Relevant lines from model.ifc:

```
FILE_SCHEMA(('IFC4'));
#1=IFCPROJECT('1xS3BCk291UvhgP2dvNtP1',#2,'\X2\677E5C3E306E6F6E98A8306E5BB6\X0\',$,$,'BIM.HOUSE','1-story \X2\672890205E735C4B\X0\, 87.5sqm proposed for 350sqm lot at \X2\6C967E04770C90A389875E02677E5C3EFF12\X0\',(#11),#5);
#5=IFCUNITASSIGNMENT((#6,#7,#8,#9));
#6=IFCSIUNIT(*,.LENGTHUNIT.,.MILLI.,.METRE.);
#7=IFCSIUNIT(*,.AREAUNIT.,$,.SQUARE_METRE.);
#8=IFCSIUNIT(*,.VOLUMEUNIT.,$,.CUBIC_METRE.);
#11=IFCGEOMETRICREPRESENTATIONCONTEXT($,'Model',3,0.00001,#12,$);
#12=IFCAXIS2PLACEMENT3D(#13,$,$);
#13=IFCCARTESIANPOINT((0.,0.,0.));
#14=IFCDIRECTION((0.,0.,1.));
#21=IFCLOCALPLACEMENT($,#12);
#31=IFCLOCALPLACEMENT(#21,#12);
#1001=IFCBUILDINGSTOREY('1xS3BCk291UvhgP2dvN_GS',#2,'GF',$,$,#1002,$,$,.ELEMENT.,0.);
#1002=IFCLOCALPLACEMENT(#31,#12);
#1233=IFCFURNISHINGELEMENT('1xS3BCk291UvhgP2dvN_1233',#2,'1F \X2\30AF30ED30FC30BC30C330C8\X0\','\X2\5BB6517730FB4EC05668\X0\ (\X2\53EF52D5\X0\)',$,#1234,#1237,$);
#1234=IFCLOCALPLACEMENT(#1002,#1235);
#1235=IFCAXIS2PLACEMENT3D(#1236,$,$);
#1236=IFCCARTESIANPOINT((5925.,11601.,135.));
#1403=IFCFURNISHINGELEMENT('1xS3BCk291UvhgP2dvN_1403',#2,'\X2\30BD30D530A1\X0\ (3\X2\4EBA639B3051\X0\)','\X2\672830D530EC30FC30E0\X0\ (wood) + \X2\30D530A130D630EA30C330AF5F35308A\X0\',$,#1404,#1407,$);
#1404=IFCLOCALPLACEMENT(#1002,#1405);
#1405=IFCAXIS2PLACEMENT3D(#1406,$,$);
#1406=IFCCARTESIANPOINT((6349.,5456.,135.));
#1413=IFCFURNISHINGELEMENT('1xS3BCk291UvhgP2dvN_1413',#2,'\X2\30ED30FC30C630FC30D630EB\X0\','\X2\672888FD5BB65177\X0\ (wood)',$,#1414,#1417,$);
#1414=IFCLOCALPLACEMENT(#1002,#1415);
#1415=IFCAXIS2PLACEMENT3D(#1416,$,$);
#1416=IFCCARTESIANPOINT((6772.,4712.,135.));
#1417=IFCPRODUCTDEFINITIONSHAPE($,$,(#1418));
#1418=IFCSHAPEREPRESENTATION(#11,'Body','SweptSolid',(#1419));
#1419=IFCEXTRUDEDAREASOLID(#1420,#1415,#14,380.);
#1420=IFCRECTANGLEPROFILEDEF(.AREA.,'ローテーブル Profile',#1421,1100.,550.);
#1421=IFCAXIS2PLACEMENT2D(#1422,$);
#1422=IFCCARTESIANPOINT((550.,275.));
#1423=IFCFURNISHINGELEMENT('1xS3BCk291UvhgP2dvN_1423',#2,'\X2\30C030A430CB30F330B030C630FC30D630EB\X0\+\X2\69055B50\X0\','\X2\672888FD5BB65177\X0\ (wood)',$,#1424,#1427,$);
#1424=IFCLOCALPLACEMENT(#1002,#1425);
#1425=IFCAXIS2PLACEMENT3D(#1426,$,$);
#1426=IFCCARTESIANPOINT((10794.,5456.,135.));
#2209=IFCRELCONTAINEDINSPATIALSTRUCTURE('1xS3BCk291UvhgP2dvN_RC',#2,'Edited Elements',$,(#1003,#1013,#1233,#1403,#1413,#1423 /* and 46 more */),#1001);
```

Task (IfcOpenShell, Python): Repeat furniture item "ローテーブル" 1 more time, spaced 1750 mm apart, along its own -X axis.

```python
import ifcopenshell
import ifcopenshell.api.geometry
import ifcopenshell.api.root
import ifcopenshell.util.element
import ifcopenshell.util.placement
import ifcopenshell.util.unit

model = ifcopenshell.open("model.ifc")
unit_scale = ifcopenshell.util.unit.calculate_unit_scale(model)


def reuse_history(source, copy):
    """copy_class also copies each property set's owner history, people and application; keep the originals."""
    for rel in copy.IsDefinedBy:
        if rel.is_a("IfcRelDefinesByProperties") and (history := rel.RelatingPropertyDefinition.OwnerHistory):
            rel.RelatingPropertyDefinition.OwnerHistory = source.OwnerHistory
            ifcopenshell.util.element.remove_deep2(model, history)


source = model.by_guid("1xS3BCk291UvhgP2dvN_1413")
base = ifcopenshell.util.placement.get_local_placement(source.ObjectPlacement)
step = -base[:3, 0] * 1.75 / unit_scale

for i in range(1, 2):
    copy = ifcopenshell.api.root.copy_class(model, product=source)
    copy.Representation = ifcopenshell.util.element.copy_deep(
        model, source.Representation, exclude=["IfcGeometricRepresentationContext", "IfcRepresentationMap"]
    )
    reuse_history(source, copy)
    matrix = base.copy()
    matrix[:3, 3] += i * step
    print("added at", matrix[:3, 3].round(3) + 0.0)
    ifcopenshell.api.geometry.edit_object_placement(model, product=copy, matrix=matrix, is_si=False)

model.write("model_edited.ifc")
```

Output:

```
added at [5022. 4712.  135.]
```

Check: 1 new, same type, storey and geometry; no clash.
